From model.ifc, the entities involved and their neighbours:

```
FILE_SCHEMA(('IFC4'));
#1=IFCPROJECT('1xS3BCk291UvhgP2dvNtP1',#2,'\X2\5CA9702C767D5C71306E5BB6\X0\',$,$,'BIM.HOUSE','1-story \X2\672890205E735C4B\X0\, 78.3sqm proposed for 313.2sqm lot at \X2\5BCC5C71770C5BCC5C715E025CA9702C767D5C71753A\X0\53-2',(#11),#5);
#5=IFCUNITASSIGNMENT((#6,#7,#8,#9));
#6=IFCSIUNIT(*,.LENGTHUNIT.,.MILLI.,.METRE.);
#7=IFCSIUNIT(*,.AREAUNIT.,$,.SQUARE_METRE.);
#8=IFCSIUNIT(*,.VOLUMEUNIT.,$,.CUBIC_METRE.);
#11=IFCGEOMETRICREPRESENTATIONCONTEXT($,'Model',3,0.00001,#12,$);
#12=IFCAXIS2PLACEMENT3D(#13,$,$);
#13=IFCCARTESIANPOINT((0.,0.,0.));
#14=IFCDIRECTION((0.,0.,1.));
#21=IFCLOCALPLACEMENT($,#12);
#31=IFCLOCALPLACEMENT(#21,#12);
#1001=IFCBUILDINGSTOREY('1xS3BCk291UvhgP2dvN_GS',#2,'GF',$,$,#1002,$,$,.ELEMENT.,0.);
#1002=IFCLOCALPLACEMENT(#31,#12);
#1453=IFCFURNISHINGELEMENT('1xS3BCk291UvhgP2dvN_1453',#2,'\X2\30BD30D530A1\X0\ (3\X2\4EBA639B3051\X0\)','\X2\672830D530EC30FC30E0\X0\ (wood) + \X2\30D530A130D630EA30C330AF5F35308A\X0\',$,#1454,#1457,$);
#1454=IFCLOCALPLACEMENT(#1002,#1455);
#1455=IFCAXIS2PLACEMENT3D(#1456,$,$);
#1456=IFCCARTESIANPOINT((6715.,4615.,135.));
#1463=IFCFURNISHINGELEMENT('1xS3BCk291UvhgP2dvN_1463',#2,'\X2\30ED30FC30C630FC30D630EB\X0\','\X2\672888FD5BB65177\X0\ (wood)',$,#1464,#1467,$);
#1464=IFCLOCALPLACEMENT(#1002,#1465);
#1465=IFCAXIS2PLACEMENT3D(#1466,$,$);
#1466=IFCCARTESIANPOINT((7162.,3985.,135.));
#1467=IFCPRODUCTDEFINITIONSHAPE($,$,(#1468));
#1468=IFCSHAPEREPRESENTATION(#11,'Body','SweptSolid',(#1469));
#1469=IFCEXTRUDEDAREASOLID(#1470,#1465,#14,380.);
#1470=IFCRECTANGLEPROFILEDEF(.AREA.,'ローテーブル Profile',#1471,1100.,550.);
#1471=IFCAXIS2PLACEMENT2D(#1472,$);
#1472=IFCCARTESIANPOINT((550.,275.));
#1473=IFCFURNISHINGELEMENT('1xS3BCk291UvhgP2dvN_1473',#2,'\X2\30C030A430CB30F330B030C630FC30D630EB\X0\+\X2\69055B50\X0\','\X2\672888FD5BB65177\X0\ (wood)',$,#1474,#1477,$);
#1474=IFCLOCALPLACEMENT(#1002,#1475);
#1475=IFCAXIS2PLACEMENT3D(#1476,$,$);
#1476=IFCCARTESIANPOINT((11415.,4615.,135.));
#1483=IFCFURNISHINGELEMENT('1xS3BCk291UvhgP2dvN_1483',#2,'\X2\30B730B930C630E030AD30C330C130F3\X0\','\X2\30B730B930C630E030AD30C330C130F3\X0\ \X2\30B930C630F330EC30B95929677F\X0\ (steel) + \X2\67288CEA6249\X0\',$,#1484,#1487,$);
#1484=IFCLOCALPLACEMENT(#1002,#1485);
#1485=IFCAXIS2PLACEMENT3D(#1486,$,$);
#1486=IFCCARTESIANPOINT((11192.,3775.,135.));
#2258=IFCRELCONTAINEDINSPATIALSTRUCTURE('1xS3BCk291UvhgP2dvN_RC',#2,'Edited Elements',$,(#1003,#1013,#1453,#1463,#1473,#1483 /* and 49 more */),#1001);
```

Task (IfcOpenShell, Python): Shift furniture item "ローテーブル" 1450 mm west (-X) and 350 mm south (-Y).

```python
import ifcopenshell
import ifcopenshell.api.geometry
import ifcopenshell.util.placement

model = ifcopenshell.open("model.ifc")

item = model.by_guid("1xS3BCk291UvhgP2dvN_1463")
matrix = ifcopenshell.util.placement.get_local_placement(item.ObjectPlacement)
matrix[0, 3] -= 1450.0
matrix[1, 3] -= 350.0
ifcopenshell.api.geometry.edit_object_placement(model, product=item, matrix=matrix, is_si=False)

print(ifcopenshell.util.placement.get_local_placement(item.ObjectPlacement).round(3) + 0.0)

model.write("model_v2.ifc")
```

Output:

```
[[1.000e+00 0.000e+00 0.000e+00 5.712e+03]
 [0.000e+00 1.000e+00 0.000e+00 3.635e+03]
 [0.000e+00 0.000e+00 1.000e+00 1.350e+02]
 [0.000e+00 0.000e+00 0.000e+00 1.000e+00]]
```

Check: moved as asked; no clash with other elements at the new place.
